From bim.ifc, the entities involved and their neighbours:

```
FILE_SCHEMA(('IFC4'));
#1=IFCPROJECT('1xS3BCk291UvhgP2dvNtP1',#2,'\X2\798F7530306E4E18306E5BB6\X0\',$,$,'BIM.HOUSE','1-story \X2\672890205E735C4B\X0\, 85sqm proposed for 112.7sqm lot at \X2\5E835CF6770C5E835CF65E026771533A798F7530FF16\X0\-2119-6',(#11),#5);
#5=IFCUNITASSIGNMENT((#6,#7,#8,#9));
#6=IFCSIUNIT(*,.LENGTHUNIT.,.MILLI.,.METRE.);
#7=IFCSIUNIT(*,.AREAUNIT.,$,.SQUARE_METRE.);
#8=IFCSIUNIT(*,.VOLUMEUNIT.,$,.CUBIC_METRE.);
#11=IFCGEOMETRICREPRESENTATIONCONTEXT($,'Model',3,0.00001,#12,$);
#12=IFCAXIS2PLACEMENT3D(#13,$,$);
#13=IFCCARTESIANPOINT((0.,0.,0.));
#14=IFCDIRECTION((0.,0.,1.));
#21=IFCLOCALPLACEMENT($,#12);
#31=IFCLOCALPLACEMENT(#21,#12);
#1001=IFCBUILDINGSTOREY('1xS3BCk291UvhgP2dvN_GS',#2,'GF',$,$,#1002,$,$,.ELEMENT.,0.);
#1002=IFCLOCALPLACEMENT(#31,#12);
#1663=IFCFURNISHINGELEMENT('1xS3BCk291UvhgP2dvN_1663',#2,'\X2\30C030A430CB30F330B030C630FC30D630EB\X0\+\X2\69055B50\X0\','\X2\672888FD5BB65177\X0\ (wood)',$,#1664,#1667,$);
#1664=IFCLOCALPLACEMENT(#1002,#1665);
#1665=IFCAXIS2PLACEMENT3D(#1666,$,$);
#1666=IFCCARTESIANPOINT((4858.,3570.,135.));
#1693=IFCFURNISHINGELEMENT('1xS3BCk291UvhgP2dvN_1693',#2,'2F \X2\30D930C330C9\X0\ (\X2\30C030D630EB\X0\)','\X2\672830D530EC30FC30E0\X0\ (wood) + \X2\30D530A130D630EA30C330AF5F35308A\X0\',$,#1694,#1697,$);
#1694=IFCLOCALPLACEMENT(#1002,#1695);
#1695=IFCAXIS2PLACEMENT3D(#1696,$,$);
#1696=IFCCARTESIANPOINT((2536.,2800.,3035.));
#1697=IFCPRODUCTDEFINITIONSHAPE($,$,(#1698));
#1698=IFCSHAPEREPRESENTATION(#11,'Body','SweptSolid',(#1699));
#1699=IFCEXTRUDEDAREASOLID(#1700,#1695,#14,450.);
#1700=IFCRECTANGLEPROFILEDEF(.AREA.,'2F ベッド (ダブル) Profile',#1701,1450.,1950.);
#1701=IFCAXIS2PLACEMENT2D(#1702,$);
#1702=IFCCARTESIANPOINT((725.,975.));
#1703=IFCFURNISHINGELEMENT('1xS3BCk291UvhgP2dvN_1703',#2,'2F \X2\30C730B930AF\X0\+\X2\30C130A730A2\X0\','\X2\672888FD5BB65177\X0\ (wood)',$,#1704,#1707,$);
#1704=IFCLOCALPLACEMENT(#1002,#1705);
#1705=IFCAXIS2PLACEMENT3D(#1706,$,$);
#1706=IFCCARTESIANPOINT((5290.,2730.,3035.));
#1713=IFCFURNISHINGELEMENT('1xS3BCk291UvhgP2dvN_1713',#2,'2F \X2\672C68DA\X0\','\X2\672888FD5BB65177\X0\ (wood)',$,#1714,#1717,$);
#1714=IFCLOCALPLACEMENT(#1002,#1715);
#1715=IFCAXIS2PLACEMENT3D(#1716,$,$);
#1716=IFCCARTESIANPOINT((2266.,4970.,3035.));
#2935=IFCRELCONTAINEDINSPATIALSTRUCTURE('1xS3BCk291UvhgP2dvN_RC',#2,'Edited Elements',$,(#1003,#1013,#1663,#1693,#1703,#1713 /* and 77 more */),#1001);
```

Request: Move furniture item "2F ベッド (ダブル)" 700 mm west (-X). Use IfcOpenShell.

```python
import ifcopenshell
import ifcopenshell.api.geometry
import ifcopenshell.util.placement

model = ifcopenshell.open("bim.ifc")

item = model.by_id(1693)
matrix = ifcopenshell.util.placement.get_local_placement(item.ObjectPlacement)
matrix[0, 3] -= 700.0
ifcopenshell.api.geometry.edit_object_placement(model, product=item, matrix=matrix, is_si=False)

print(ifcopenshell.util.placement.get_local_placement(item.ObjectPlacement).round(3) + 0.0)

model.write("bim_rev.ifc")
```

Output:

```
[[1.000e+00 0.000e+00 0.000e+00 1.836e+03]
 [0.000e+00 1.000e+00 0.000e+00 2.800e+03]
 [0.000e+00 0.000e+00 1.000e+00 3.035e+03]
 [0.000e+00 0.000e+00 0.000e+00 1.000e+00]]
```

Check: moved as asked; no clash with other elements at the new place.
